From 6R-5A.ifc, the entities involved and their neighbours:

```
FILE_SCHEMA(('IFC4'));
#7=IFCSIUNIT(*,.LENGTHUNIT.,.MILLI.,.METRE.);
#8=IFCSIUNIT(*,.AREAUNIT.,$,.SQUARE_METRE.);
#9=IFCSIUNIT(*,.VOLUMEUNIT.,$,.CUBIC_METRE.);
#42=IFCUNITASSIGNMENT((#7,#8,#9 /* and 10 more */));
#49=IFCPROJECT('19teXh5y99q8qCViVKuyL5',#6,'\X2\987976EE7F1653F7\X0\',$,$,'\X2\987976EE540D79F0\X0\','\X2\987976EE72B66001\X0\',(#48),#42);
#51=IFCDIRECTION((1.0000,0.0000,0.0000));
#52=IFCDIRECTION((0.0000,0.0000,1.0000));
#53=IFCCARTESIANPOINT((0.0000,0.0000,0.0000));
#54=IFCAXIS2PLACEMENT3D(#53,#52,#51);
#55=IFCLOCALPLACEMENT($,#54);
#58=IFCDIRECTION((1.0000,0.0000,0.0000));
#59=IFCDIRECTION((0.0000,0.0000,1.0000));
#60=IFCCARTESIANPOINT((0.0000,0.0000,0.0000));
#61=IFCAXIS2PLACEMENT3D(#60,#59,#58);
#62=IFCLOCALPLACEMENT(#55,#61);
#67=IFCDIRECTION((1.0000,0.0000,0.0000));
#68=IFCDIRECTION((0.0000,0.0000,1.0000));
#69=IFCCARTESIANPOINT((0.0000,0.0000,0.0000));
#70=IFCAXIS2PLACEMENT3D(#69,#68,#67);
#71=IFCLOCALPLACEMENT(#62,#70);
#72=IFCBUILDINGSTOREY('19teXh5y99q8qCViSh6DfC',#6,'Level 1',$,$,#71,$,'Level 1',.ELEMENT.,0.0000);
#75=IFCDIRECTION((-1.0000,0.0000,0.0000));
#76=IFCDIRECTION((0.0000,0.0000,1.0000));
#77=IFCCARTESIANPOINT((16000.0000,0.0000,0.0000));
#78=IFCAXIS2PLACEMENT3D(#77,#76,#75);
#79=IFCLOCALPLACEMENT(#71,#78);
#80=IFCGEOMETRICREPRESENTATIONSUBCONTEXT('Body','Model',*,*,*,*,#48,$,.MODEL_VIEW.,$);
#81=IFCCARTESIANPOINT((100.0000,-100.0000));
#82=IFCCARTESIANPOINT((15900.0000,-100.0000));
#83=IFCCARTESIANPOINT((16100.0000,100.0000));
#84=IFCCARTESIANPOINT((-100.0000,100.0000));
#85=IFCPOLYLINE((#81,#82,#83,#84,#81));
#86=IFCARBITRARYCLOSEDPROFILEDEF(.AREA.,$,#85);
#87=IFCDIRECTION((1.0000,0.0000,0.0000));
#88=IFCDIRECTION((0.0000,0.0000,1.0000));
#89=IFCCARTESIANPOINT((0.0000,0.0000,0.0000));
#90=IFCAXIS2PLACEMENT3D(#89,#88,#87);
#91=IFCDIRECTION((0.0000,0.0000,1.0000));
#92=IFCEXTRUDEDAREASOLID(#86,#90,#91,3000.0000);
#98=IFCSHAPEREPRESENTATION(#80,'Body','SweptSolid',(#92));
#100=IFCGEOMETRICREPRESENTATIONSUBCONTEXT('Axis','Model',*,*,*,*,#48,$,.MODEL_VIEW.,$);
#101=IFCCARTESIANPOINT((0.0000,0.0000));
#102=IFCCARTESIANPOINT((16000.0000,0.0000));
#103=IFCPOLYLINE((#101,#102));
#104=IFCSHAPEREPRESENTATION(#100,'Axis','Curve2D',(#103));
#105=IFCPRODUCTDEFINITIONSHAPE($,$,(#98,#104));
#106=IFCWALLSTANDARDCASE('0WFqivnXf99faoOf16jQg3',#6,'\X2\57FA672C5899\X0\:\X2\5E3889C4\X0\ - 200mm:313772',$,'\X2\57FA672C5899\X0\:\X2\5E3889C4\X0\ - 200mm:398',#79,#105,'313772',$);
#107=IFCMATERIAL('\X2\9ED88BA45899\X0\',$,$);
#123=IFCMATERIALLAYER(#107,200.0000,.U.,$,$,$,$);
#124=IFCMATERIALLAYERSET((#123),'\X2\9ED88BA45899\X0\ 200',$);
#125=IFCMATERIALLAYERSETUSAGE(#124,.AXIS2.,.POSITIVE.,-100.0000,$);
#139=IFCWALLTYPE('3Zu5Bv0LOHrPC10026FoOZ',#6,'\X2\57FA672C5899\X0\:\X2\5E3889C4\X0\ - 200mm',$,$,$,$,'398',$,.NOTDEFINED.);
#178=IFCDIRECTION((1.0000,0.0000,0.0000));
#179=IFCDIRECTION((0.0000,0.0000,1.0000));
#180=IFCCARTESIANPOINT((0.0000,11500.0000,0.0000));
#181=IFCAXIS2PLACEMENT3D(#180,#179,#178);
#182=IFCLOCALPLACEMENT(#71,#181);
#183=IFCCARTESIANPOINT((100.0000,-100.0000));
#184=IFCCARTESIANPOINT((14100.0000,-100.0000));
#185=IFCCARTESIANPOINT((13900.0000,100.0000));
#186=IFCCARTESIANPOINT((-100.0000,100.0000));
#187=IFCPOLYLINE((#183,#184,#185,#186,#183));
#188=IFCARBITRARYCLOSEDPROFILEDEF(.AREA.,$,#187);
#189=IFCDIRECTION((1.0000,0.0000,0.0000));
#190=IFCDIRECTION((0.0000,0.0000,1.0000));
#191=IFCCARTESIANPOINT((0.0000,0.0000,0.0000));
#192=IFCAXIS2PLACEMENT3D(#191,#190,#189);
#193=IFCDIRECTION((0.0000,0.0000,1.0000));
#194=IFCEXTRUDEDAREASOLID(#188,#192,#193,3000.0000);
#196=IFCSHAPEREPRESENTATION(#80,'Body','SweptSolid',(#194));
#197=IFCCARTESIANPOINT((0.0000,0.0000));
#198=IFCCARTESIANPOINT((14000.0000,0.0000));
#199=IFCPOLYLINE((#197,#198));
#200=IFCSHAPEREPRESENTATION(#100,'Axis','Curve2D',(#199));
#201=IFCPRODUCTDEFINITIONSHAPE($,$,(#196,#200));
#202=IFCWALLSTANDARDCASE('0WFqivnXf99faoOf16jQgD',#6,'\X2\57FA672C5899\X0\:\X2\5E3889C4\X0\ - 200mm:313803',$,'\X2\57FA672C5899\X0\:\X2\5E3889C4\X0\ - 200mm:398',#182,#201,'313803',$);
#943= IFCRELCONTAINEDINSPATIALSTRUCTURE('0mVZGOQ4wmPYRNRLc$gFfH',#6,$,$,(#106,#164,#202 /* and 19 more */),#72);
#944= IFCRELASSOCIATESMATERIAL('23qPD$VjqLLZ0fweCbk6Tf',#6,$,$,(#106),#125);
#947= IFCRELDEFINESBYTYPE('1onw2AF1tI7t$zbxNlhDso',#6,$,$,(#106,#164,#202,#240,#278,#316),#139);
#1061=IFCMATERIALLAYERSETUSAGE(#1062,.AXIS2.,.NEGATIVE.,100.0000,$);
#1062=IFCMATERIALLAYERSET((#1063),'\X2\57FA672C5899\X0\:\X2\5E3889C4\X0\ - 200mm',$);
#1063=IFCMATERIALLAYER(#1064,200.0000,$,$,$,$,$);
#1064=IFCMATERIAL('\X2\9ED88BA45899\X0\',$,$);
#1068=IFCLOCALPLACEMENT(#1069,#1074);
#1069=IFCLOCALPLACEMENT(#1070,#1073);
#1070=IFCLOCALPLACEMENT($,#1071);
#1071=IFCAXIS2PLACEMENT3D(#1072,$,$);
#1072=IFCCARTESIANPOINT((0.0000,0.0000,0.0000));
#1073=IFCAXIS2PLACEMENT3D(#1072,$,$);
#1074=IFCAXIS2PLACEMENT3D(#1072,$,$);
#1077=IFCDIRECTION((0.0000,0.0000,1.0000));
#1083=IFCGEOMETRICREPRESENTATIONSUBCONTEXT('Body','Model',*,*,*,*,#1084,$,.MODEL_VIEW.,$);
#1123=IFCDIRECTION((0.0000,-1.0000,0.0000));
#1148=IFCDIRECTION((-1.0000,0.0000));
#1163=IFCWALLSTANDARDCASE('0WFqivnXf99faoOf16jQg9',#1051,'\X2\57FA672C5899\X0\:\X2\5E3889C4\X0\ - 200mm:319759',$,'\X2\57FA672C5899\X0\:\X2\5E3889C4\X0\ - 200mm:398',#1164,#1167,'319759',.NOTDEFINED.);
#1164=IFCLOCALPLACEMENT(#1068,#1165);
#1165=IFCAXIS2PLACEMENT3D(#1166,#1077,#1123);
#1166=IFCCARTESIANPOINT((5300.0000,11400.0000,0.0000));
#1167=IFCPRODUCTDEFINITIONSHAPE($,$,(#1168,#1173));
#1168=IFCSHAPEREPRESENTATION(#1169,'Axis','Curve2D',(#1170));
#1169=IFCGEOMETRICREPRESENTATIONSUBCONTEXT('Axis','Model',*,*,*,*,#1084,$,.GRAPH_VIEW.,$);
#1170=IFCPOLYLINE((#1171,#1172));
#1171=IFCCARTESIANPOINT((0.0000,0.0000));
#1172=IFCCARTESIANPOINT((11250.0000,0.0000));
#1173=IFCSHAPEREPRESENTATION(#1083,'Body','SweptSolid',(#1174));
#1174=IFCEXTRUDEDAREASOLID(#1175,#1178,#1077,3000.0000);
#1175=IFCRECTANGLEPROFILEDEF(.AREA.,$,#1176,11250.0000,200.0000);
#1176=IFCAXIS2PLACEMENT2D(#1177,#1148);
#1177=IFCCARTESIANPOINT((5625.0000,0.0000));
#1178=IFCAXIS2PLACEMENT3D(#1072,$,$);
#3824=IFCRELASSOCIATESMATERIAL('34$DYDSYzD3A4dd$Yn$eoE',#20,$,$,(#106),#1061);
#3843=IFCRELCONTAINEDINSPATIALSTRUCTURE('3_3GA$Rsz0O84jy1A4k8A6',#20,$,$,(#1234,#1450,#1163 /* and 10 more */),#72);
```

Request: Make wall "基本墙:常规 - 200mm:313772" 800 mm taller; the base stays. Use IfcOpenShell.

```python
import ifcopenshell
import ifcopenshell.geom
import ifcopenshell.util.representation
import ifcopenshell.util.shape

model = ifcopenshell.open("6R-5A.ifc")
settings = ifcopenshell.geom.settings()


def volume(element):
    """Net volume in cubic metres, openings subtracted."""
    shape = ifcopenshell.geom.create_shape(settings, element)
    return ifcopenshell.util.shape.get_volume(shape.geometry)


wall = model.by_id(106)
before = volume(wall)

body = ifcopenshell.util.representation.get_representation(wall, "Model", "Body")
solid = body.Items[0]
old_height = solid.Depth
solid.Depth += 800.0
after = volume(wall)

print(f"height {old_height:g} -> {solid.Depth:g}, volume {before:.3f} -> {after:.3f} m3")

model.write("6R-5A_updated.ifc")
```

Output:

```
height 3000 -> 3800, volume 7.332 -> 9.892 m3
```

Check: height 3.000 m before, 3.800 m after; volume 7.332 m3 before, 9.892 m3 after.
